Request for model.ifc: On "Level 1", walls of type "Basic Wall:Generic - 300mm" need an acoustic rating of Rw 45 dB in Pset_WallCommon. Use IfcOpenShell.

First a look at what the model holds.

```python
import ifcopenshell
import ifcopenshell.util.element

model = ifcopenshell.open("model.ifc")
print(model.schema)
storey = next(s for s in model.by_type("IfcBuildingStorey") if s.Name == "Level 1")
walls = [e for e in ifcopenshell.util.element.get_decomposition(storey) if e.is_a("IfcWall")]
seen = {}
for e in walls:
    element_type = ifcopenshell.util.element.get_type(e)
    key = (element_type.Name if element_type != e and element_type else None, ifcopenshell.util.element.get_pset(e, "Pset_WallCommon", "AcousticRating"))
    seen[key] = seen.get(key, 0) + 1
for (name, value), count in sorted(seen.items(), key=str):
    print(count, "x", name, "|", value)
```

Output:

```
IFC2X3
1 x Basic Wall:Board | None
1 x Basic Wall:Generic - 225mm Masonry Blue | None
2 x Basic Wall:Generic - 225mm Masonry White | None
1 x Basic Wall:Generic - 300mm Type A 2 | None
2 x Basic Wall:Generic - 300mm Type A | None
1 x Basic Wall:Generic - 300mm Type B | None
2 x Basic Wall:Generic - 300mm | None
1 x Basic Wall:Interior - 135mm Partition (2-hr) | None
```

```python
import ifcopenshell
import ifcopenshell.api.pset
import ifcopenshell.util.element

model = ifcopenshell.open("model.ifc")

storey = next(s for s in model.by_type("IfcBuildingStorey") if s.Name == "Level 1")
walls = [e for e in ifcopenshell.util.element.get_decomposition(storey) if e.is_a("IfcWall")]

count = 0
for e in walls:
    element_type = ifcopenshell.util.element.get_type(e)
    if element_type in (None, e) or element_type.Name != "Basic Wall:Generic - 300mm":
        continue
    # add_pset returns the element's existing set when there is one.
    pset = ifcopenshell.api.pset.add_pset(model, product=e, name="Pset_WallCommon")
    ifcopenshell.api.pset.edit_pset(model, pset=pset, properties={"AcousticRating": "Rw 45 dB"})
    count += 1

print(count, "walls updated")

model.write("model_v2.ifc")
```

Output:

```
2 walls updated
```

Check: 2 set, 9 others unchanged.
